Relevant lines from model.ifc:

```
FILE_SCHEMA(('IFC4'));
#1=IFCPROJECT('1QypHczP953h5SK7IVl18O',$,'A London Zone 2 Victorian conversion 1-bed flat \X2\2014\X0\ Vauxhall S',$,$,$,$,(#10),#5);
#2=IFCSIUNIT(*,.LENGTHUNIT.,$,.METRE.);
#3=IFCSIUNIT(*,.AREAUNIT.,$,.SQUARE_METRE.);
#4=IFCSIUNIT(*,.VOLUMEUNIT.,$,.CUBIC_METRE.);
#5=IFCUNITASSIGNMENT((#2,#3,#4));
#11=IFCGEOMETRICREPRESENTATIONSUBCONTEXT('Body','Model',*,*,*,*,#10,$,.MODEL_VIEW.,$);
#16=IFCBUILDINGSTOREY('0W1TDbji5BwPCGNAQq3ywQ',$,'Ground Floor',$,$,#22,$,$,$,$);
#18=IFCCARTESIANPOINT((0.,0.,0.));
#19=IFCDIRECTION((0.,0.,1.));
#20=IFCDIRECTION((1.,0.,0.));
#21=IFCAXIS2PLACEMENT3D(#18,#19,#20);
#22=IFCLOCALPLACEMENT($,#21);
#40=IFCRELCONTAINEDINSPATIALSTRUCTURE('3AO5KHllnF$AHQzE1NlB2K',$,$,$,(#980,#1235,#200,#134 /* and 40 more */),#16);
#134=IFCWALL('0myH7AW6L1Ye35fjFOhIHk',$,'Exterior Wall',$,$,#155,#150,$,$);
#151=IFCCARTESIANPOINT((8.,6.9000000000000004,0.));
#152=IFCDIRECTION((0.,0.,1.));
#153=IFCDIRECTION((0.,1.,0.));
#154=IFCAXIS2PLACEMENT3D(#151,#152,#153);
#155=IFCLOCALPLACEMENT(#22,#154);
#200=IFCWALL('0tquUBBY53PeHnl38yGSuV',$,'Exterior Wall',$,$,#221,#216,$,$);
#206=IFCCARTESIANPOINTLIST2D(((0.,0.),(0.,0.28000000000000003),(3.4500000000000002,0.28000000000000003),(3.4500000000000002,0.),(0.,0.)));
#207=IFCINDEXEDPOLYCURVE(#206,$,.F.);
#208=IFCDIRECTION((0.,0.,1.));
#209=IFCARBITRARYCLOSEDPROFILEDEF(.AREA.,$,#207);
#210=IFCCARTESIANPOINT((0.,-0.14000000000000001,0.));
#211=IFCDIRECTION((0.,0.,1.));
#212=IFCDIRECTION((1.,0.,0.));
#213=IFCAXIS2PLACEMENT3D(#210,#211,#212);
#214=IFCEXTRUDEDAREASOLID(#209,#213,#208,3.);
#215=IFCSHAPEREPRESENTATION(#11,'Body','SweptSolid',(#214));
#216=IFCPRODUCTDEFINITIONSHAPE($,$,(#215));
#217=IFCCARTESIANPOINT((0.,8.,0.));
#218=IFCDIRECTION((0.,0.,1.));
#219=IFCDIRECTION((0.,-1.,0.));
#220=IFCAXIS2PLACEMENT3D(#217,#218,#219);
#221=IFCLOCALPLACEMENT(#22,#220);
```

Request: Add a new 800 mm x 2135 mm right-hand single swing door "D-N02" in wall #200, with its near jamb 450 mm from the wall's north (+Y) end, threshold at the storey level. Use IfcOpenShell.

```python
import numpy as np
import ifcopenshell
import ifcopenshell.api.feature
import ifcopenshell.api.geometry
import ifcopenshell.api.root
import ifcopenshell.api.spatial
import ifcopenshell.geom
import ifcopenshell.util.element
import ifcopenshell.util.placement
import ifcopenshell.util.representation
import ifcopenshell.util.shape
import ifcopenshell.util.unit

model = ifcopenshell.open("model.ifc")
unit_scale = ifcopenshell.util.unit.calculate_unit_scale(model)
settings = ifcopenshell.geom.settings()


def volume(element):
    """Net volume in cubic metres, openings subtracted."""
    shape = ifcopenshell.geom.create_shape(settings, element)
    return ifcopenshell.util.shape.get_volume(shape.geometry)


wall = model.by_guid("0tquUBBY53PeHnl38yGSuV")
storey = ifcopenshell.util.element.get_container(wall, ifc_class="IfcBuildingStorey")
context = ifcopenshell.util.representation.get_context(model, "Model", "Body", "MODEL_VIEW")
before = volume(wall)

width, height, from_end, sill = 0.8, 2.135, 0.45, 0.0  # metres

# The wall runs along its own X axis, and the end named is its -X end.
wall_shape = ifcopenshell.geom.create_shape(settings, wall)
x, y, z = ifcopenshell.util.shape.get_vertices(wall_shape.geometry).T
start = x.min() + from_end
face, thickness = float(y.min()), float(y.max() - y.min())
wall_matrix = ifcopenshell.util.placement.get_local_placement(wall.ObjectPlacement)
level = ifcopenshell.util.placement.get_local_placement(storey.ObjectPlacement)[2, 3]


def in_wall(x, y):
    """Placement at x, y metres in the wall's axes, at sill height."""
    matrix = wall_matrix.copy()
    matrix[:, 3] = wall_matrix @ np.array([x / unit_scale, y / unit_scale, 0.0, 1.0])
    matrix[2, 3] = level + sill / unit_scale
    return matrix


# Opening: a box that overshoots both wall faces by 50 mm.
opening = ifcopenshell.api.root.create_entity(model, ifc_class="IfcOpeningElement", predefined_type="OPENING")
box = ifcopenshell.api.geometry.add_wall_representation(
    model, context=context, length=width, height=height, thickness=thickness + 0.1
)
ifcopenshell.api.geometry.assign_representation(model, product=opening, representation=box)
ifcopenshell.api.geometry.edit_object_placement(model, product=opening, matrix=in_wall(start, face - 0.05), is_si=False)
ifcopenshell.api.feature.add_feature(model, feature=opening, element=wall)

door = ifcopenshell.api.root.create_entity(model, ifc_class="IfcDoor", name="D-N02", predefined_type="DOOR")
door.OverallWidth, door.OverallHeight = width / unit_scale, height / unit_scale
door.OperationType = "SINGLE_SWING_RIGHT"
body = ifcopenshell.api.geometry.add_door_representation(
    model,
    context=context,
    overall_width=door.OverallWidth,
    overall_height=door.OverallHeight,
    operation_type="SINGLE_SWING_RIGHT",
    lining_properties={"LiningDepth": thickness / unit_scale, "ThresholdDepth": thickness / unit_scale},
)
ifcopenshell.api.geometry.assign_representation(model, product=door, representation=body)
ifcopenshell.api.spatial.assign_container(model, products=[door], relating_structure=storey)
ifcopenshell.api.feature.add_filling(model, opening=opening, element=door)

# The lining spans the wall, so the door starts at the wall face.
ifcopenshell.api.geometry.edit_object_placement(model, product=door, matrix=in_wall(start, face), is_si=False)

after = volume(wall)

print(f"wall volume {before:.3f} -> {after:.3f} m3")

model.write("model_v2.ifc")
```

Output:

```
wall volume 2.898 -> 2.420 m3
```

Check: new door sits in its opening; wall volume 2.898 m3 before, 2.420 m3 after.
